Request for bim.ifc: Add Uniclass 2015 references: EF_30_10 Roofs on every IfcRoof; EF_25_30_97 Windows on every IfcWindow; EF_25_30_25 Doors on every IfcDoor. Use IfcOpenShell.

First a look at what the model holds.

```python
import ifcopenshell

model = ifcopenshell.open("bim.ifc")
print(model.schema)
print("classifications:", [c.Name for c in model.by_type("IfcClassification")])
for ifc_class in ("IfcDoor", "IfcRoof", "IfcStair", "IfcWall", "IfcWindow"):
    print(ifc_class, len(model.by_type(ifc_class)))
```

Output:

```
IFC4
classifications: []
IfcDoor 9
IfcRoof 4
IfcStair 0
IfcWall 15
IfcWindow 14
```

```python
import ifcopenshell
import ifcopenshell.api.classification

model = ifcopenshell.open("bim.ifc")

system = ifcopenshell.api.classification.add_classification(model, classification="Uniclass 2015")

codes = {
    "IfcRoof": ("EF_30_10", "Roofs"),
    "IfcWindow": ("EF_25_30_97", "Windows"),
    "IfcDoor": ("EF_25_30_25", "Doors"),
}
for ifc_class, (code, name) in codes.items():
    products = model.by_type(ifc_class)
    ifcopenshell.api.classification.add_reference(
        model, products=products, classification=system, identification=code, name=name
    )
    print(code, len(products))

model.write("bim_updated.ifc")
```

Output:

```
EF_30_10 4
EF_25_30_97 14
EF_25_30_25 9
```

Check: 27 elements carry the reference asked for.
